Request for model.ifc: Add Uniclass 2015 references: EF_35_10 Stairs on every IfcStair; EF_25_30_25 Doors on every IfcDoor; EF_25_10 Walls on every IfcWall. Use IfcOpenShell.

First a look at what the model holds.

```python
import ifcopenshell

model = ifcopenshell.open("model.ifc")
print(model.schema)
print("classifications:", [c.Name for c in model.by_type("IfcClassification")])
for ifc_class in ("IfcDoor", "IfcRoof", "IfcStair", "IfcWall", "IfcWindow"):
    print(ifc_class, len(model.by_type(ifc_class)))
```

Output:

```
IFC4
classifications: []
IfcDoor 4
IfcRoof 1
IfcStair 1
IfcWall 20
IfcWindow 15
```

```python
import ifcopenshell
import ifcopenshell.api.classification

model = ifcopenshell.open("model.ifc")

system = ifcopenshell.api.classification.add_classification(model, classification="Uniclass 2015")

codes = {
    "IfcStair": ("EF_35_10", "Stairs"),
    "IfcDoor": ("EF_25_30_25", "Doors"),
    "IfcWall": ("EF_25_10", "Walls"),
}
for ifc_class, (code, name) in codes.items():
    products = model.by_type(ifc_class)
    ifcopenshell.api.classification.add_reference(
        model, products=products, classification=system, identification=code, name=name
    )
    print(code, len(products))

model.write("model_edited.ifc")
```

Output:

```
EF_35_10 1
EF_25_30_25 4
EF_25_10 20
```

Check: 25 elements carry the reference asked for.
